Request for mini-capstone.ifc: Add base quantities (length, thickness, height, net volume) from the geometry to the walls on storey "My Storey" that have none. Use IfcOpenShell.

First a look at what the model holds.

```python
import ifcopenshell
import ifcopenshell.util.element
import ifcopenshell.util.unit

model = ifcopenshell.open("mini-capstone.ifc")
print(model.schema)
for unit_type in ("LENGTHUNIT", "AREAUNIT", "VOLUMEUNIT"):
    print(unit_type, ifcopenshell.util.unit.calculate_unit_scale(model, unit_type))
storey = next(s for s in model.by_type("IfcBuildingStorey") if s.Name == "My Storey")
walls = [e for e in ifcopenshell.util.element.get_decomposition(storey) if e.is_a("IfcWall")]
for e in sorted(walls, key=lambda e: e.id()):
    print(e.id(), e.is_a(), e.Name, list(ifcopenshell.util.element.get_psets(e, qtos_only=True)), sep=" | ")
```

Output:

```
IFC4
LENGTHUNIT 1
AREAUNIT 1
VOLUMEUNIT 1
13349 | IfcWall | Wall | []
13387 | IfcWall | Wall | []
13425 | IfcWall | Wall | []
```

```python
import ifcopenshell
import ifcopenshell.api.pset
import ifcopenshell.geom
import ifcopenshell.util.element
import ifcopenshell.util.shape
import ifcopenshell.util.unit

model = ifcopenshell.open("mini-capstone.ifc")
unit_scale = ifcopenshell.util.unit.calculate_unit_scale(model)
volume_scale = ifcopenshell.util.unit.calculate_unit_scale(model, "VOLUMEUNIT")
settings = ifcopenshell.geom.settings()

storey = next(s for s in model.by_type("IfcBuildingStorey") if s.Name == "My Storey")
walls = [e for e in ifcopenshell.util.element.get_decomposition(storey) if e.is_a("IfcWall")]

for e in sorted(walls, key=lambda e: e.id()):
    if ifcopenshell.util.element.get_psets(e, qtos_only=True, should_inherit=False):
        continue
    # Geometry comes back in metres, in the element's own axes.
    shape = ifcopenshell.geom.create_shape(settings, e)
    values = {
        "Length": ifcopenshell.util.shape.get_x(shape.geometry) / unit_scale,
        "Width": ifcopenshell.util.shape.get_y(shape.geometry) / unit_scale,
        "Height": ifcopenshell.util.shape.get_z(shape.geometry) / unit_scale,
        "NetVolume": ifcopenshell.util.shape.get_volume(shape.geometry) / volume_scale,
    }
    qto = ifcopenshell.api.pset.add_qto(model, product=e, name="Qto_WallBaseQuantities")
    ifcopenshell.api.pset.edit_qto(model, qto=qto, properties=values)
    print(e.id(), {k: round(v, 3) for k, v in values.items()})

model.write("mini-capstone_v2.ifc")
```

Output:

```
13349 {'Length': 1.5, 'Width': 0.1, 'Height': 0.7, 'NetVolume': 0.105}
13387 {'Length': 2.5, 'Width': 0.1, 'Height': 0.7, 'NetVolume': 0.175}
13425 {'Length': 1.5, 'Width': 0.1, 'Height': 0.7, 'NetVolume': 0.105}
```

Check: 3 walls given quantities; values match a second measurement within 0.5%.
